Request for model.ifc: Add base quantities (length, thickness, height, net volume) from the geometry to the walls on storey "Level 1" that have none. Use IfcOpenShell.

First a look at what the model holds.

```python
import ifcopenshell
import ifcopenshell.util.element
import ifcopenshell.util.unit

model = ifcopenshell.open("model.ifc")
print(model.schema)
for unit_type in ("LENGTHUNIT", "AREAUNIT", "VOLUMEUNIT"):
    print(unit_type, ifcopenshell.util.unit.calculate_unit_scale(model, unit_type))
storey = next(s for s in model.by_type("IfcBuildingStorey") if s.Name == "Level 1")
walls = [e for e in ifcopenshell.util.element.get_decomposition(storey) if e.is_a("IfcWall")]
for e in sorted(walls, key=lambda e: e.id()):
    print(e.id(), e.is_a(), e.Name, list(ifcopenshell.util.element.get_psets(e, qtos_only=True)), sep=" | ")
```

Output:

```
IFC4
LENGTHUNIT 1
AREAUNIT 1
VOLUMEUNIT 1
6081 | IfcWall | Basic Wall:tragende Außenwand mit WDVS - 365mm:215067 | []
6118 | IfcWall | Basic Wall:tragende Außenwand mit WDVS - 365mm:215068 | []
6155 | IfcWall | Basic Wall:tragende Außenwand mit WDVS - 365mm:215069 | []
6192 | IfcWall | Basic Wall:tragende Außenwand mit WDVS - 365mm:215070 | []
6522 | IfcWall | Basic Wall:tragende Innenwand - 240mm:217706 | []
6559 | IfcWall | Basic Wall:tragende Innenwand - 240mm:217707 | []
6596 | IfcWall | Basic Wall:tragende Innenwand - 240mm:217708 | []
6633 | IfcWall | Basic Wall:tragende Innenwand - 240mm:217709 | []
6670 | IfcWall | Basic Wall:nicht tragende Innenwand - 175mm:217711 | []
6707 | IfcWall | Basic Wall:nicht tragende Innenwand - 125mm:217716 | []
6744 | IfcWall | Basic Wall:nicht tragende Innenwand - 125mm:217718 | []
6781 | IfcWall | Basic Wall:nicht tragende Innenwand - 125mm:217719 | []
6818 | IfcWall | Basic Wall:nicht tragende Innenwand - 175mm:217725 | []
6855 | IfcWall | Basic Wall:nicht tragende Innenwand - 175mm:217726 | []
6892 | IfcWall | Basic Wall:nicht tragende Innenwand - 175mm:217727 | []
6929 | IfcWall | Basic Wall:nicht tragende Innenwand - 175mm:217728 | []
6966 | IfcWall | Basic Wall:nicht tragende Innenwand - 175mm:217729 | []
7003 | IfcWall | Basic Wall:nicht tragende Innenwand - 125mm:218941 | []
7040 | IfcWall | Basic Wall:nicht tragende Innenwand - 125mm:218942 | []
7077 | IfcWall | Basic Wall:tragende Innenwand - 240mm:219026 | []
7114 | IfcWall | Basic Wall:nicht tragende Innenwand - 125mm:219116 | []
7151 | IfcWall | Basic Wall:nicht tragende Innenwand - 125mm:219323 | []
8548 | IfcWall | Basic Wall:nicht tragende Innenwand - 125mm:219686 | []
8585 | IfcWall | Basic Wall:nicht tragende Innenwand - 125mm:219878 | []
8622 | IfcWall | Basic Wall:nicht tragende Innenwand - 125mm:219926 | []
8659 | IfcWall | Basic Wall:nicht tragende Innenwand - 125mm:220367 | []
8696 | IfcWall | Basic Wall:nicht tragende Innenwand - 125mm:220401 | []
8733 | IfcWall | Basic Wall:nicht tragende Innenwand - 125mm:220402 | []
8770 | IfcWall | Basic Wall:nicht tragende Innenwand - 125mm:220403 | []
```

```python
import ifcopenshell
import ifcopenshell.api.pset
import ifcopenshell.geom
import ifcopenshell.util.element
import ifcopenshell.util.shape
import ifcopenshell.util.unit

model = ifcopenshell.open("model.ifc")
unit_scale = ifcopenshell.util.unit.calculate_unit_scale(model)
volume_scale = ifcopenshell.util.unit.calculate_unit_scale(model, "VOLUMEUNIT")
settings = ifcopenshell.geom.settings()

storey = next(s for s in model.by_type("IfcBuildingStorey") if s.Name == "Level 1")
walls = [e for e in ifcopenshell.util.element.get_decomposition(storey) if e.is_a("IfcWall")]

for e in sorted(walls, key=lambda e: e.id()):
    if ifcopenshell.util.element.get_psets(e, qtos_only=True, should_inherit=False):
        continue
    # Geometry comes back in metres, in the element's own axes.
    shape = ifcopenshell.geom.create_shape(settings, e)
    values = {
        "Length": ifcopenshell.util.shape.get_x(shape.geometry) / unit_scale,
        "Width": ifcopenshell.util.shape.get_y(shape.geometry) / unit_scale,
        "Height": ifcopenshell.util.shape.get_z(shape.geometry) / unit_scale,
        "NetVolume": ifcopenshell.util.shape.get_volume(shape.geometry) / volume_scale,
    }
    qto = ifcopenshell.api.pset.add_qto(model, product=e, name="Qto_WallBaseQuantities")
    ifcopenshell.api.pset.edit_qto(model, qto=qto, properties=values)
    print(e.id(), {k: round(v, 3) for k, v in values.items()})

model.write("model_edited.ifc")
```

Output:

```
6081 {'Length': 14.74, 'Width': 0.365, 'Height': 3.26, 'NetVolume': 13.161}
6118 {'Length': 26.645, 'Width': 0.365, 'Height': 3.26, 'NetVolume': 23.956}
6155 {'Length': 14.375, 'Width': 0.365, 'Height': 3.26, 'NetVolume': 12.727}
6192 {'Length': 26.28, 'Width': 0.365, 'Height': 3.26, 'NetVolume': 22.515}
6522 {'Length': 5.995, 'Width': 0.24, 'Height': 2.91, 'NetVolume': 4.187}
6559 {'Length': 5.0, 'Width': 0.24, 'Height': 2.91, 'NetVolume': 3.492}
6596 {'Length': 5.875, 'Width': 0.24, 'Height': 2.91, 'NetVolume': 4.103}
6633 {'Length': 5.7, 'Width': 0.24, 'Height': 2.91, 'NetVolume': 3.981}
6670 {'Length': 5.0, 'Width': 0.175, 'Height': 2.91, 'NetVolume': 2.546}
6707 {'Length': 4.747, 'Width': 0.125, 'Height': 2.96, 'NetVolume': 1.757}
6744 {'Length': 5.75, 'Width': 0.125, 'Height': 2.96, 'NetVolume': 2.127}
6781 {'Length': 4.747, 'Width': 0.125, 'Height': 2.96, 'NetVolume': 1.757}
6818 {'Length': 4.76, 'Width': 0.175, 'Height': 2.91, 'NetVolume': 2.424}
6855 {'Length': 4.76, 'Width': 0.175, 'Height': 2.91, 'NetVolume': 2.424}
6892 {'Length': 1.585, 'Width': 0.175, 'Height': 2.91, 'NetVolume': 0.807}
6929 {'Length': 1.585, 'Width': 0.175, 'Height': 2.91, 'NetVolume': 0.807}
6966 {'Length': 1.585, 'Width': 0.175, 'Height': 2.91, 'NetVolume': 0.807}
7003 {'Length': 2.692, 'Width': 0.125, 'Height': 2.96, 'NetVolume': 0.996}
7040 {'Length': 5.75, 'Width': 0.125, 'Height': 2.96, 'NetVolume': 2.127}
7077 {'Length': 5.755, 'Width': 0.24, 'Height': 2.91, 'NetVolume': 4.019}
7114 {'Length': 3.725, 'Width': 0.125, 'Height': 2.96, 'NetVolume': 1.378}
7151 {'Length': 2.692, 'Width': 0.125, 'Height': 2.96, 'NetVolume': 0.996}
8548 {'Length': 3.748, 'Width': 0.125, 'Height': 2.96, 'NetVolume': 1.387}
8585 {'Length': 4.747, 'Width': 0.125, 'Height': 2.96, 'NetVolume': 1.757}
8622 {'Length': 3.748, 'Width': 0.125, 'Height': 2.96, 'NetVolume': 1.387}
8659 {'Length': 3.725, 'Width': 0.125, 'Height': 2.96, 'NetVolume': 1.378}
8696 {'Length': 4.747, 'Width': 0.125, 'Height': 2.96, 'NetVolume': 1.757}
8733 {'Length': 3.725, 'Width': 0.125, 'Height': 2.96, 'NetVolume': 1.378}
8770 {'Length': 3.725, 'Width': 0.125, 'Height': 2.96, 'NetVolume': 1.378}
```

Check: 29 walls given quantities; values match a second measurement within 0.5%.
